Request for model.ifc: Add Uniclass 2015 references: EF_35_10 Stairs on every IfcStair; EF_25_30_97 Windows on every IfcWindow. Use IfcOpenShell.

First a look at what the model holds.

```python
import ifcopenshell

model = ifcopenshell.open("model.ifc")
print(model.schema)
print("classifications:", [c.Name for c in model.by_type("IfcClassification")])
for ifc_class in ("IfcDoor", "IfcRoof", "IfcStair", "IfcWall", "IfcWindow"):
    print(ifc_class, len(model.by_type(ifc_class)))
```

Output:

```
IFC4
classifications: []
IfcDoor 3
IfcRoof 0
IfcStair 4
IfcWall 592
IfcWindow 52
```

```python
import ifcopenshell
import ifcopenshell.api.classification

model = ifcopenshell.open("model.ifc")

system = ifcopenshell.api.classification.add_classification(model, classification="Uniclass 2015")

codes = {
    "IfcStair": ("EF_35_10", "Stairs"),
    "IfcWindow": ("EF_25_30_97", "Windows"),
}
for ifc_class, (code, name) in codes.items():
    products = model.by_type(ifc_class)
    ifcopenshell.api.classification.add_reference(
        model, products=products, classification=system, identification=code, name=name
    )
    print(code, len(products))

model.write("model_v2.ifc")
```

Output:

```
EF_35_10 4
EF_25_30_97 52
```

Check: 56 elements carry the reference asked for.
